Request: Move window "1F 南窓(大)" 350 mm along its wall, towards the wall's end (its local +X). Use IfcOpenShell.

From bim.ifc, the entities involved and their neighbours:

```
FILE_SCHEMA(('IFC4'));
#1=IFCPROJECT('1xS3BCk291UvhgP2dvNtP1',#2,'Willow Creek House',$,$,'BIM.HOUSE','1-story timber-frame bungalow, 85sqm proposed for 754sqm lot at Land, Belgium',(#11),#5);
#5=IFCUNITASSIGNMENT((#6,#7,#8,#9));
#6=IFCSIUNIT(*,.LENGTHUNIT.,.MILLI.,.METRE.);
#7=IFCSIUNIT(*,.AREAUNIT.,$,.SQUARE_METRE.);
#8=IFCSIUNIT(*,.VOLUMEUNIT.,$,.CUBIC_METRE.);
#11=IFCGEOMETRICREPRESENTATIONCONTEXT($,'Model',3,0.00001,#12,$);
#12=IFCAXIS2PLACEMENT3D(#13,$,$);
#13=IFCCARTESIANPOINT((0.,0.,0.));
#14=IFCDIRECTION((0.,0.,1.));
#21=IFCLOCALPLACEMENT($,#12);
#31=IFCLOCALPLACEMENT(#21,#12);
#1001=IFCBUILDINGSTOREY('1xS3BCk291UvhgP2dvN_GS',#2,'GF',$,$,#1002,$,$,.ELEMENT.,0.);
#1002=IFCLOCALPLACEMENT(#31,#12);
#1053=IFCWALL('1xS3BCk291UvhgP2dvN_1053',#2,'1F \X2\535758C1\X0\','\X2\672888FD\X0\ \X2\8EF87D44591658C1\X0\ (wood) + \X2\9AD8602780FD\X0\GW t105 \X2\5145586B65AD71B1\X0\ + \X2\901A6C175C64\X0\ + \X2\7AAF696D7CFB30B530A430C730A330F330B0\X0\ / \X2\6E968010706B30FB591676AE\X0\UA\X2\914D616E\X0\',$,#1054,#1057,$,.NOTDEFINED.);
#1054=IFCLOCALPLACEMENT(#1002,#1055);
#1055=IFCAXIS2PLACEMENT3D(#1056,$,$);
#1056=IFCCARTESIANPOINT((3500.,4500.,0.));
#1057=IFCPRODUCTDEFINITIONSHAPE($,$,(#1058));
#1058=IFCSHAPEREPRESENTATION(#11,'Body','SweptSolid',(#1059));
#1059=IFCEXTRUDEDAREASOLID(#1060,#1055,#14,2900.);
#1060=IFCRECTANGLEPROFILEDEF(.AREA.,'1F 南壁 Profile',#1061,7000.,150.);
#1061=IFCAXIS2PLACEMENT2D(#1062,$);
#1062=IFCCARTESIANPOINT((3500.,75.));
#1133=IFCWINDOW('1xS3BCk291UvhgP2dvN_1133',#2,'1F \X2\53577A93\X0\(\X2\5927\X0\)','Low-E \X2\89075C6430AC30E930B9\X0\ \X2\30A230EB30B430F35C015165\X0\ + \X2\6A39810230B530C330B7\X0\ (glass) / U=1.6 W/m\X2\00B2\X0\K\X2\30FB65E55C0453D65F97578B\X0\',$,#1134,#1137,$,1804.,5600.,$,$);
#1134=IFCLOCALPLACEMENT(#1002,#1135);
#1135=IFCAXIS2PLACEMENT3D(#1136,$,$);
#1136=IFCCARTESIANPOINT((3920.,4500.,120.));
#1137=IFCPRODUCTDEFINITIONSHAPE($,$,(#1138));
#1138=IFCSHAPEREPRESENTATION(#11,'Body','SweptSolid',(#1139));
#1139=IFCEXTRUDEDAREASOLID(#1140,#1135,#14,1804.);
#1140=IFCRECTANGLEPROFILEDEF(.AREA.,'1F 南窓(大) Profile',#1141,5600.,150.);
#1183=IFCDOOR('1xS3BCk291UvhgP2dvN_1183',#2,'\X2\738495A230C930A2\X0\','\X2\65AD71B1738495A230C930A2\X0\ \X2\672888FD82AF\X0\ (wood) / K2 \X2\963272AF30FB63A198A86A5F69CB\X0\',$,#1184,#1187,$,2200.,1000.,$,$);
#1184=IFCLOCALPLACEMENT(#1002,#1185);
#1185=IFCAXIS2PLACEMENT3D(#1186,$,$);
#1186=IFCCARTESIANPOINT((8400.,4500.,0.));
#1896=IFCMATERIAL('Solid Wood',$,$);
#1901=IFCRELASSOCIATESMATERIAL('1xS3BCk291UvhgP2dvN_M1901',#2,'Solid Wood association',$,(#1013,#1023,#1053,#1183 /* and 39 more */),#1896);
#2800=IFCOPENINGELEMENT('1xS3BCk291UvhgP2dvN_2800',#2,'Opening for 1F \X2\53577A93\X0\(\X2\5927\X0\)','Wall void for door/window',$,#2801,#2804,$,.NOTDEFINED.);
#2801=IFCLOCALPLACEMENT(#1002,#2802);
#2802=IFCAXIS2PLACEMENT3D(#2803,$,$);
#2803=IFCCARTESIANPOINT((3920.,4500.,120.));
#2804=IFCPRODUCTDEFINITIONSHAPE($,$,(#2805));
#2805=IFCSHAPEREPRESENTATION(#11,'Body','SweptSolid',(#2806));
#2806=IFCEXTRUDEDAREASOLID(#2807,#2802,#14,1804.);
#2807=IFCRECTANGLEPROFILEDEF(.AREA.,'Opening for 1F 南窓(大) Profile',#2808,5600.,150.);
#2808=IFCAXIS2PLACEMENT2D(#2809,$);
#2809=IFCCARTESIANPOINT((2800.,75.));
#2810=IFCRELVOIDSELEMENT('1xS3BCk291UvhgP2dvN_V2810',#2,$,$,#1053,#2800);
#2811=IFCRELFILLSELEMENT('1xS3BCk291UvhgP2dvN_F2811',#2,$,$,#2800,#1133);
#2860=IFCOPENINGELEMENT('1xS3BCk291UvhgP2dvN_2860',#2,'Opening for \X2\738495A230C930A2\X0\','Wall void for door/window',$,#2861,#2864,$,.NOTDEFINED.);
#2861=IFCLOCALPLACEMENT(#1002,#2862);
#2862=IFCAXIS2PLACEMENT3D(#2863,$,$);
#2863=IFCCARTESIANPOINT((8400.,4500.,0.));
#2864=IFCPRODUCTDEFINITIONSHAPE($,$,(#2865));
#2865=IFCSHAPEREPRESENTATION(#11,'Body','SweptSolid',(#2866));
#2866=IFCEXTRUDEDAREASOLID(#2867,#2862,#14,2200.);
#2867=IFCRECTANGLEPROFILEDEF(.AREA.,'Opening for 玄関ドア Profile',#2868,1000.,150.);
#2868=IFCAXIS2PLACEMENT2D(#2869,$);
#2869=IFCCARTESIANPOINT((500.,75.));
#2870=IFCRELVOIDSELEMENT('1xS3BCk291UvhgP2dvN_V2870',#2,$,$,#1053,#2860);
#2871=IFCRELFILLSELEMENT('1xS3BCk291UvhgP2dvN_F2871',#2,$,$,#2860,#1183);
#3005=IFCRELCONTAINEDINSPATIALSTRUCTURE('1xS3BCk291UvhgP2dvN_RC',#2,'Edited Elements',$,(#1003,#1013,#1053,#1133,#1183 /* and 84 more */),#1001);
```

```python
import ifcopenshell
import ifcopenshell.api.geometry
import ifcopenshell.util.placement

model = ifcopenshell.open("bim.ifc")

window = model.by_id(1133)
opening = window.FillsVoids[0].RelatingOpeningElement
wall = opening.VoidsElements[0].RelatingBuildingElement

wall_matrix = ifcopenshell.util.placement.get_local_placement(wall.ObjectPlacement)
shift = wall_matrix[:3, 0] * 350.0
before = ifcopenshell.util.placement.get_local_placement(window.ObjectPlacement)[:3, 3].copy()

# The window is not placed relative to its opening, so move both.
for product in (opening, window):
    matrix = ifcopenshell.util.placement.get_local_placement(product.ObjectPlacement)
    matrix[:3, 3] += shift
    ifcopenshell.api.geometry.edit_object_placement(model, product=product, matrix=matrix, is_si=False)

after = ifcopenshell.util.placement.get_local_placement(window.ObjectPlacement)[:3, 3]
print("window moved by", (after - before).round(3) + 0.0)

model.write("bim_rev.ifc")
```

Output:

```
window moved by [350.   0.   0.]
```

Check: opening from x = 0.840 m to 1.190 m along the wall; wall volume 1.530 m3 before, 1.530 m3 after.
